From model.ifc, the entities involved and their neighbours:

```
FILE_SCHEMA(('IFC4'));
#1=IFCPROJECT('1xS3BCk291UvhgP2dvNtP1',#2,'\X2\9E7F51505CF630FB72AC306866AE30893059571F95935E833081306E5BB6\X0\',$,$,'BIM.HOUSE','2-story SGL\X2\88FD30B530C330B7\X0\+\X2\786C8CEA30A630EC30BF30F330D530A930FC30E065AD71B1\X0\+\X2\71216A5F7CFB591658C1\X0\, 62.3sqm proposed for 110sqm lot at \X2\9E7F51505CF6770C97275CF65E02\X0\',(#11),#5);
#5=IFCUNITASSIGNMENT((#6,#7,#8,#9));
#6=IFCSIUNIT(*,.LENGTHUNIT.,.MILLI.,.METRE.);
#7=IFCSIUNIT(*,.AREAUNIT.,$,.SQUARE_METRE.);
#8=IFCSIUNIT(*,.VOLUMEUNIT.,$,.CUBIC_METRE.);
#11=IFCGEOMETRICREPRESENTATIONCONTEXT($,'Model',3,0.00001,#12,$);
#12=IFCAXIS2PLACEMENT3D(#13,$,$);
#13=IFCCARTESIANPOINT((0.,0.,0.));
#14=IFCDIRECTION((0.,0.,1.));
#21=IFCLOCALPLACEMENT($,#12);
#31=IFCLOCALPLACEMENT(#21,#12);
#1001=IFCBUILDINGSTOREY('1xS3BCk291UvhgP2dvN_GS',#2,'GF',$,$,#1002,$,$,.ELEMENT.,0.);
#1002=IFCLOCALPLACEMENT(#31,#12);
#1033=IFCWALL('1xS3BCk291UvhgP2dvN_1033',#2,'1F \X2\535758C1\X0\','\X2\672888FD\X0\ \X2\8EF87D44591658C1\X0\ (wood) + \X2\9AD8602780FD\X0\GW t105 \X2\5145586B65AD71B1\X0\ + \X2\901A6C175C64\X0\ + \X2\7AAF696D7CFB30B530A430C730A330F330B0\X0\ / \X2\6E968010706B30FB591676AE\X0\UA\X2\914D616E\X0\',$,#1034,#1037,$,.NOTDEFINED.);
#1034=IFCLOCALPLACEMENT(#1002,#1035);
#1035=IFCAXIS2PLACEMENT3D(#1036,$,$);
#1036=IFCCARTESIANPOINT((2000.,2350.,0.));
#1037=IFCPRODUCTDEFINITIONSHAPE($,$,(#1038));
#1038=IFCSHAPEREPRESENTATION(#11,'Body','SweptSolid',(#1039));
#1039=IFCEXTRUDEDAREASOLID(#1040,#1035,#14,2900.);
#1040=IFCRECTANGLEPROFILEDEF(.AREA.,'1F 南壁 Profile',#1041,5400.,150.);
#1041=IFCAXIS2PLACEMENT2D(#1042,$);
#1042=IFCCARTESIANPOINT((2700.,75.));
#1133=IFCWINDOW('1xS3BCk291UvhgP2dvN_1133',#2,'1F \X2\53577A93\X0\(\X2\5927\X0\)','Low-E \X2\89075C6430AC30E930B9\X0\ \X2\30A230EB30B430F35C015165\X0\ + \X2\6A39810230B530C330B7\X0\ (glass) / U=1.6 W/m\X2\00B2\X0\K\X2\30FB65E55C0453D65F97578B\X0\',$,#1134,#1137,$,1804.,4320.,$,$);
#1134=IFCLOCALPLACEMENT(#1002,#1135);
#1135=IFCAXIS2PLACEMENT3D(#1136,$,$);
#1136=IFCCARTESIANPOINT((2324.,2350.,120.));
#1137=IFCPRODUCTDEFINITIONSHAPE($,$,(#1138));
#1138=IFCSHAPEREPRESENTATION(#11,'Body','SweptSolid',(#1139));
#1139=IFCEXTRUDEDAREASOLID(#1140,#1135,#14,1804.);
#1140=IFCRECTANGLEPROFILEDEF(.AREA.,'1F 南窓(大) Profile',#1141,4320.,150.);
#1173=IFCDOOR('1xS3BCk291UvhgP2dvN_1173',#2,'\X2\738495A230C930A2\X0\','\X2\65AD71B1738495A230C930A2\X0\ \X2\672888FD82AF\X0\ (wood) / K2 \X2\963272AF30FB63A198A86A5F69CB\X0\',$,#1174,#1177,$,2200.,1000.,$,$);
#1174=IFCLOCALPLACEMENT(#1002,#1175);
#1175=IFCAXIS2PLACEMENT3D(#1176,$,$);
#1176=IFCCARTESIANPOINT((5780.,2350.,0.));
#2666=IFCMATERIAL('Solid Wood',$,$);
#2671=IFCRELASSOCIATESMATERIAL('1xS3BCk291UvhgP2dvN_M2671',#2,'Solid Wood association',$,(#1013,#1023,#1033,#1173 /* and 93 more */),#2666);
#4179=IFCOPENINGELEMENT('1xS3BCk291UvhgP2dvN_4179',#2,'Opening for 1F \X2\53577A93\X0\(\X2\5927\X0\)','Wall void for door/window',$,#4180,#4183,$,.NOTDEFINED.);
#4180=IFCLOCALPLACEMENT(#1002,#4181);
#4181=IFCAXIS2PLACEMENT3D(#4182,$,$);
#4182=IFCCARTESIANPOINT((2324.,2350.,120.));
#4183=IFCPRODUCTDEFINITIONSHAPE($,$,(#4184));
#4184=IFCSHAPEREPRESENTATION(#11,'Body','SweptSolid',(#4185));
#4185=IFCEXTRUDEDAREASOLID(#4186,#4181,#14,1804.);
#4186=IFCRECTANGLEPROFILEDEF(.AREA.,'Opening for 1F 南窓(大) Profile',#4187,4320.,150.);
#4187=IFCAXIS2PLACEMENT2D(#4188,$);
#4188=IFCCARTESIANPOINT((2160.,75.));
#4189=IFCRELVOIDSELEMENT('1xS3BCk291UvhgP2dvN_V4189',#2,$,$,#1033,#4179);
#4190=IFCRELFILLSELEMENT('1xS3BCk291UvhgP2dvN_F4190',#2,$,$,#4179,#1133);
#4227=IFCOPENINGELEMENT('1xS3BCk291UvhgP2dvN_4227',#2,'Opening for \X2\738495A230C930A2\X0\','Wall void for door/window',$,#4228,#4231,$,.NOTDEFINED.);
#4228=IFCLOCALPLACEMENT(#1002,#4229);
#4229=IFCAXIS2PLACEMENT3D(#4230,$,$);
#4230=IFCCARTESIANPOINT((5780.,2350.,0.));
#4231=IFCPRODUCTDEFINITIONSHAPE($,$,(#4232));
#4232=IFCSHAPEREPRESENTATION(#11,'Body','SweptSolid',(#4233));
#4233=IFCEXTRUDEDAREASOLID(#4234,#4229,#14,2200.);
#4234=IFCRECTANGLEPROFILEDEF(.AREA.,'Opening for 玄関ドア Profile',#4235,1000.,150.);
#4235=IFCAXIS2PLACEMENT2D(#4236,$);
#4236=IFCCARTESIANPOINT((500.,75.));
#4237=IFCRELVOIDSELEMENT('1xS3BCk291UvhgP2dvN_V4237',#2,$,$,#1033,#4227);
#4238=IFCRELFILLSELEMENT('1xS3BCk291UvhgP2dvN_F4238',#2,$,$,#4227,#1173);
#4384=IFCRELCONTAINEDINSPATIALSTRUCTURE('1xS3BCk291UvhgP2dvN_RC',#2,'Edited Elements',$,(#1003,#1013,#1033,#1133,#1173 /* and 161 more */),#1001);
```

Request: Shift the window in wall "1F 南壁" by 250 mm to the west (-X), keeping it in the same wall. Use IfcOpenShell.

```python
import ifcopenshell
import ifcopenshell.api.geometry
import ifcopenshell.util.placement

model = ifcopenshell.open("model.ifc")

window = model.by_guid("1xS3BCk291UvhgP2dvN_1133")
opening = window.FillsVoids[0].RelatingOpeningElement
wall = opening.VoidsElements[0].RelatingBuildingElement

wall_matrix = ifcopenshell.util.placement.get_local_placement(wall.ObjectPlacement)
shift = wall_matrix[:3, 0] * -250.0
before = ifcopenshell.util.placement.get_local_placement(window.ObjectPlacement)[:3, 3].copy()

# The window is not placed relative to its opening, so move both.
for product in (opening, window):
    matrix = ifcopenshell.util.placement.get_local_placement(product.ObjectPlacement)
    matrix[:3, 3] += shift
    ifcopenshell.api.geometry.edit_object_placement(model, product=product, matrix=matrix, is_si=False)

after = ifcopenshell.util.placement.get_local_placement(window.ObjectPlacement)[:3, 3]
print("window moved by", (after - before).round(3) + 0.0)

model.write("model_rev.ifc")
```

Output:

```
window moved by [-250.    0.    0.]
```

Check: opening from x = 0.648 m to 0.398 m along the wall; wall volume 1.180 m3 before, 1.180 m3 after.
